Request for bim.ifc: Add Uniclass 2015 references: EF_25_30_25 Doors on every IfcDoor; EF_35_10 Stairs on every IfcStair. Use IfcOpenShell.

First a look at what the model holds.

```python
import ifcopenshell

model = ifcopenshell.open("bim.ifc")
print(model.schema)
print("classifications:", [c.Name for c in model.by_type("IfcClassification")])
for ifc_class in ("IfcDoor", "IfcRoof", "IfcStair", "IfcWall", "IfcWindow"):
    print(ifc_class, len(model.by_type(ifc_class)))
```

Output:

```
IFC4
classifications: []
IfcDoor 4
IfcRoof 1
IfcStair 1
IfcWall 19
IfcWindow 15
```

```python
import ifcopenshell
import ifcopenshell.api.classification

model = ifcopenshell.open("bim.ifc")

system = ifcopenshell.api.classification.add_classification(model, classification="Uniclass 2015")

codes = {
    "IfcDoor": ("EF_25_30_25", "Doors"),
    "IfcStair": ("EF_35_10", "Stairs"),
}
for ifc_class, (code, name) in codes.items():
    products = model.by_type(ifc_class)
    ifcopenshell.api.classification.add_reference(
        model, products=products, classification=system, identification=code, name=name
    )
    print(code, len(products))

model.write("bim_rev.ifc")
```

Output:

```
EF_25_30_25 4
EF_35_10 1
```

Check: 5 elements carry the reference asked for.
